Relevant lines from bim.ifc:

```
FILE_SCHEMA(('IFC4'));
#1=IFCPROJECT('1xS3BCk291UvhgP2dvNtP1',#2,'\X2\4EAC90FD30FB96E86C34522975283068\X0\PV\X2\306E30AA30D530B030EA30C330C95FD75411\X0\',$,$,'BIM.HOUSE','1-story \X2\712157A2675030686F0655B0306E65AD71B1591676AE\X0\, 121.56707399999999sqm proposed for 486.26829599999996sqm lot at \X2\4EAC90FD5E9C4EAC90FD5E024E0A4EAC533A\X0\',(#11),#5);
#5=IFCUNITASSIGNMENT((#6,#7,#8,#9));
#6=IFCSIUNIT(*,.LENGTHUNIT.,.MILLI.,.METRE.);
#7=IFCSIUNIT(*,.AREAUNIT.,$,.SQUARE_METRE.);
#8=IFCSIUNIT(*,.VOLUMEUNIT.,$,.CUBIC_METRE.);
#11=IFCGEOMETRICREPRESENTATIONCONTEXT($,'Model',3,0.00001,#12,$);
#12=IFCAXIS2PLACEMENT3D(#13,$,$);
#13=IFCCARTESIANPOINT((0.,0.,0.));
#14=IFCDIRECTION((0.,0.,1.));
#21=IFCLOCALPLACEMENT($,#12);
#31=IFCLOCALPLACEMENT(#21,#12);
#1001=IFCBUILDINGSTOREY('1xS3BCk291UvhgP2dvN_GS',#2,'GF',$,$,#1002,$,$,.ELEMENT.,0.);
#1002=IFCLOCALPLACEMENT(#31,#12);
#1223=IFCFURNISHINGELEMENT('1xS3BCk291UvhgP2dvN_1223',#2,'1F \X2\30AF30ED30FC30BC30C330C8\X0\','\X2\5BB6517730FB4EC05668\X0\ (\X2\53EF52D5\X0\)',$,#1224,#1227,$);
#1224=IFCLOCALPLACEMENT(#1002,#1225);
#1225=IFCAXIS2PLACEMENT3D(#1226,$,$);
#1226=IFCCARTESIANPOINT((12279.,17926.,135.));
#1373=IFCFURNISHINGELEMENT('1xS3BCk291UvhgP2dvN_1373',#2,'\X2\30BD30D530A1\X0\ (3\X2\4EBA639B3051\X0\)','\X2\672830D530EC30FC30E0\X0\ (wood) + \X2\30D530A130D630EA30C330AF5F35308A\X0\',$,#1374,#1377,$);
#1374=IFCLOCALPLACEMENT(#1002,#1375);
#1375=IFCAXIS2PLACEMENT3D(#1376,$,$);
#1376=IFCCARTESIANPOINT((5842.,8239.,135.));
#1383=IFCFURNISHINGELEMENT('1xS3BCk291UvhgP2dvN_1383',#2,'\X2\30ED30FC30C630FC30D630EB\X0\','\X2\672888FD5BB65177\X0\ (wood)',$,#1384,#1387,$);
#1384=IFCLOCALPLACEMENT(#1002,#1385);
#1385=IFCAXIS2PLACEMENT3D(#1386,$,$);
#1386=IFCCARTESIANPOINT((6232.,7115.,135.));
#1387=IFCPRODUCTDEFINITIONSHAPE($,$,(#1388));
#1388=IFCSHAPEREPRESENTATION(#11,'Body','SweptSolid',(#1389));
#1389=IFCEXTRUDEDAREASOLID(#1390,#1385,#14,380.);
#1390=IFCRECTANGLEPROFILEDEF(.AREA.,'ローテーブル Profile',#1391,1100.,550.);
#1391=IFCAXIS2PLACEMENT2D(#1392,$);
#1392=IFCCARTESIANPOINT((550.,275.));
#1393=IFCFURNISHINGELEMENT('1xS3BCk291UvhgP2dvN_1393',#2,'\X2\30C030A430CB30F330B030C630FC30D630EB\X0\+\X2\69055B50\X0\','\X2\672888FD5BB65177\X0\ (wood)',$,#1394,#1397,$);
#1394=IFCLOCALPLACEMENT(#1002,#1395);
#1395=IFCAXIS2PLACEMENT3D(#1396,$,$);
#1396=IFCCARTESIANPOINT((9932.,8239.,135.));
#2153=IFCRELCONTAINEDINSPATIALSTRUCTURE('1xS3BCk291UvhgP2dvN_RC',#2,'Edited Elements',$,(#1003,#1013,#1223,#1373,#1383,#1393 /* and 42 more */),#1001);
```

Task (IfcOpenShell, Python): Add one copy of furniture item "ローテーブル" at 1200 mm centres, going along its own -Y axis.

```python
import ifcopenshell
import ifcopenshell.api.geometry
import ifcopenshell.api.root
import ifcopenshell.util.element
import ifcopenshell.util.placement
import ifcopenshell.util.unit

model = ifcopenshell.open("bim.ifc")
unit_scale = ifcopenshell.util.unit.calculate_unit_scale(model)


def reuse_history(source, copy):
    """copy_class also copies each property set's owner history, people and application; keep the originals."""
    for rel in copy.IsDefinedBy:
        if rel.is_a("IfcRelDefinesByProperties") and (history := rel.RelatingPropertyDefinition.OwnerHistory):
            rel.RelatingPropertyDefinition.OwnerHistory = source.OwnerHistory
            ifcopenshell.util.element.remove_deep2(model, history)


source = model.by_guid("1xS3BCk291UvhgP2dvN_1383")
base = ifcopenshell.util.placement.get_local_placement(source.ObjectPlacement)
step = -base[:3, 1] * 1.2 / unit_scale

for i in range(1, 2):
    copy = ifcopenshell.api.root.copy_class(model, product=source)
    copy.Representation = ifcopenshell.util.element.copy_deep(
        model, source.Representation, exclude=["IfcGeometricRepresentationContext", "IfcRepresentationMap"]
    )
    reuse_history(source, copy)
    matrix = base.copy()
    matrix[:3, 3] += i * step
    print("added at", matrix[:3, 3].round(3) + 0.0)
    ifcopenshell.api.geometry.edit_object_placement(model, product=copy, matrix=matrix, is_si=False)

model.write("bim_v2.ifc")
```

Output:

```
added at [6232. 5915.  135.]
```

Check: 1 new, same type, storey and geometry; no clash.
